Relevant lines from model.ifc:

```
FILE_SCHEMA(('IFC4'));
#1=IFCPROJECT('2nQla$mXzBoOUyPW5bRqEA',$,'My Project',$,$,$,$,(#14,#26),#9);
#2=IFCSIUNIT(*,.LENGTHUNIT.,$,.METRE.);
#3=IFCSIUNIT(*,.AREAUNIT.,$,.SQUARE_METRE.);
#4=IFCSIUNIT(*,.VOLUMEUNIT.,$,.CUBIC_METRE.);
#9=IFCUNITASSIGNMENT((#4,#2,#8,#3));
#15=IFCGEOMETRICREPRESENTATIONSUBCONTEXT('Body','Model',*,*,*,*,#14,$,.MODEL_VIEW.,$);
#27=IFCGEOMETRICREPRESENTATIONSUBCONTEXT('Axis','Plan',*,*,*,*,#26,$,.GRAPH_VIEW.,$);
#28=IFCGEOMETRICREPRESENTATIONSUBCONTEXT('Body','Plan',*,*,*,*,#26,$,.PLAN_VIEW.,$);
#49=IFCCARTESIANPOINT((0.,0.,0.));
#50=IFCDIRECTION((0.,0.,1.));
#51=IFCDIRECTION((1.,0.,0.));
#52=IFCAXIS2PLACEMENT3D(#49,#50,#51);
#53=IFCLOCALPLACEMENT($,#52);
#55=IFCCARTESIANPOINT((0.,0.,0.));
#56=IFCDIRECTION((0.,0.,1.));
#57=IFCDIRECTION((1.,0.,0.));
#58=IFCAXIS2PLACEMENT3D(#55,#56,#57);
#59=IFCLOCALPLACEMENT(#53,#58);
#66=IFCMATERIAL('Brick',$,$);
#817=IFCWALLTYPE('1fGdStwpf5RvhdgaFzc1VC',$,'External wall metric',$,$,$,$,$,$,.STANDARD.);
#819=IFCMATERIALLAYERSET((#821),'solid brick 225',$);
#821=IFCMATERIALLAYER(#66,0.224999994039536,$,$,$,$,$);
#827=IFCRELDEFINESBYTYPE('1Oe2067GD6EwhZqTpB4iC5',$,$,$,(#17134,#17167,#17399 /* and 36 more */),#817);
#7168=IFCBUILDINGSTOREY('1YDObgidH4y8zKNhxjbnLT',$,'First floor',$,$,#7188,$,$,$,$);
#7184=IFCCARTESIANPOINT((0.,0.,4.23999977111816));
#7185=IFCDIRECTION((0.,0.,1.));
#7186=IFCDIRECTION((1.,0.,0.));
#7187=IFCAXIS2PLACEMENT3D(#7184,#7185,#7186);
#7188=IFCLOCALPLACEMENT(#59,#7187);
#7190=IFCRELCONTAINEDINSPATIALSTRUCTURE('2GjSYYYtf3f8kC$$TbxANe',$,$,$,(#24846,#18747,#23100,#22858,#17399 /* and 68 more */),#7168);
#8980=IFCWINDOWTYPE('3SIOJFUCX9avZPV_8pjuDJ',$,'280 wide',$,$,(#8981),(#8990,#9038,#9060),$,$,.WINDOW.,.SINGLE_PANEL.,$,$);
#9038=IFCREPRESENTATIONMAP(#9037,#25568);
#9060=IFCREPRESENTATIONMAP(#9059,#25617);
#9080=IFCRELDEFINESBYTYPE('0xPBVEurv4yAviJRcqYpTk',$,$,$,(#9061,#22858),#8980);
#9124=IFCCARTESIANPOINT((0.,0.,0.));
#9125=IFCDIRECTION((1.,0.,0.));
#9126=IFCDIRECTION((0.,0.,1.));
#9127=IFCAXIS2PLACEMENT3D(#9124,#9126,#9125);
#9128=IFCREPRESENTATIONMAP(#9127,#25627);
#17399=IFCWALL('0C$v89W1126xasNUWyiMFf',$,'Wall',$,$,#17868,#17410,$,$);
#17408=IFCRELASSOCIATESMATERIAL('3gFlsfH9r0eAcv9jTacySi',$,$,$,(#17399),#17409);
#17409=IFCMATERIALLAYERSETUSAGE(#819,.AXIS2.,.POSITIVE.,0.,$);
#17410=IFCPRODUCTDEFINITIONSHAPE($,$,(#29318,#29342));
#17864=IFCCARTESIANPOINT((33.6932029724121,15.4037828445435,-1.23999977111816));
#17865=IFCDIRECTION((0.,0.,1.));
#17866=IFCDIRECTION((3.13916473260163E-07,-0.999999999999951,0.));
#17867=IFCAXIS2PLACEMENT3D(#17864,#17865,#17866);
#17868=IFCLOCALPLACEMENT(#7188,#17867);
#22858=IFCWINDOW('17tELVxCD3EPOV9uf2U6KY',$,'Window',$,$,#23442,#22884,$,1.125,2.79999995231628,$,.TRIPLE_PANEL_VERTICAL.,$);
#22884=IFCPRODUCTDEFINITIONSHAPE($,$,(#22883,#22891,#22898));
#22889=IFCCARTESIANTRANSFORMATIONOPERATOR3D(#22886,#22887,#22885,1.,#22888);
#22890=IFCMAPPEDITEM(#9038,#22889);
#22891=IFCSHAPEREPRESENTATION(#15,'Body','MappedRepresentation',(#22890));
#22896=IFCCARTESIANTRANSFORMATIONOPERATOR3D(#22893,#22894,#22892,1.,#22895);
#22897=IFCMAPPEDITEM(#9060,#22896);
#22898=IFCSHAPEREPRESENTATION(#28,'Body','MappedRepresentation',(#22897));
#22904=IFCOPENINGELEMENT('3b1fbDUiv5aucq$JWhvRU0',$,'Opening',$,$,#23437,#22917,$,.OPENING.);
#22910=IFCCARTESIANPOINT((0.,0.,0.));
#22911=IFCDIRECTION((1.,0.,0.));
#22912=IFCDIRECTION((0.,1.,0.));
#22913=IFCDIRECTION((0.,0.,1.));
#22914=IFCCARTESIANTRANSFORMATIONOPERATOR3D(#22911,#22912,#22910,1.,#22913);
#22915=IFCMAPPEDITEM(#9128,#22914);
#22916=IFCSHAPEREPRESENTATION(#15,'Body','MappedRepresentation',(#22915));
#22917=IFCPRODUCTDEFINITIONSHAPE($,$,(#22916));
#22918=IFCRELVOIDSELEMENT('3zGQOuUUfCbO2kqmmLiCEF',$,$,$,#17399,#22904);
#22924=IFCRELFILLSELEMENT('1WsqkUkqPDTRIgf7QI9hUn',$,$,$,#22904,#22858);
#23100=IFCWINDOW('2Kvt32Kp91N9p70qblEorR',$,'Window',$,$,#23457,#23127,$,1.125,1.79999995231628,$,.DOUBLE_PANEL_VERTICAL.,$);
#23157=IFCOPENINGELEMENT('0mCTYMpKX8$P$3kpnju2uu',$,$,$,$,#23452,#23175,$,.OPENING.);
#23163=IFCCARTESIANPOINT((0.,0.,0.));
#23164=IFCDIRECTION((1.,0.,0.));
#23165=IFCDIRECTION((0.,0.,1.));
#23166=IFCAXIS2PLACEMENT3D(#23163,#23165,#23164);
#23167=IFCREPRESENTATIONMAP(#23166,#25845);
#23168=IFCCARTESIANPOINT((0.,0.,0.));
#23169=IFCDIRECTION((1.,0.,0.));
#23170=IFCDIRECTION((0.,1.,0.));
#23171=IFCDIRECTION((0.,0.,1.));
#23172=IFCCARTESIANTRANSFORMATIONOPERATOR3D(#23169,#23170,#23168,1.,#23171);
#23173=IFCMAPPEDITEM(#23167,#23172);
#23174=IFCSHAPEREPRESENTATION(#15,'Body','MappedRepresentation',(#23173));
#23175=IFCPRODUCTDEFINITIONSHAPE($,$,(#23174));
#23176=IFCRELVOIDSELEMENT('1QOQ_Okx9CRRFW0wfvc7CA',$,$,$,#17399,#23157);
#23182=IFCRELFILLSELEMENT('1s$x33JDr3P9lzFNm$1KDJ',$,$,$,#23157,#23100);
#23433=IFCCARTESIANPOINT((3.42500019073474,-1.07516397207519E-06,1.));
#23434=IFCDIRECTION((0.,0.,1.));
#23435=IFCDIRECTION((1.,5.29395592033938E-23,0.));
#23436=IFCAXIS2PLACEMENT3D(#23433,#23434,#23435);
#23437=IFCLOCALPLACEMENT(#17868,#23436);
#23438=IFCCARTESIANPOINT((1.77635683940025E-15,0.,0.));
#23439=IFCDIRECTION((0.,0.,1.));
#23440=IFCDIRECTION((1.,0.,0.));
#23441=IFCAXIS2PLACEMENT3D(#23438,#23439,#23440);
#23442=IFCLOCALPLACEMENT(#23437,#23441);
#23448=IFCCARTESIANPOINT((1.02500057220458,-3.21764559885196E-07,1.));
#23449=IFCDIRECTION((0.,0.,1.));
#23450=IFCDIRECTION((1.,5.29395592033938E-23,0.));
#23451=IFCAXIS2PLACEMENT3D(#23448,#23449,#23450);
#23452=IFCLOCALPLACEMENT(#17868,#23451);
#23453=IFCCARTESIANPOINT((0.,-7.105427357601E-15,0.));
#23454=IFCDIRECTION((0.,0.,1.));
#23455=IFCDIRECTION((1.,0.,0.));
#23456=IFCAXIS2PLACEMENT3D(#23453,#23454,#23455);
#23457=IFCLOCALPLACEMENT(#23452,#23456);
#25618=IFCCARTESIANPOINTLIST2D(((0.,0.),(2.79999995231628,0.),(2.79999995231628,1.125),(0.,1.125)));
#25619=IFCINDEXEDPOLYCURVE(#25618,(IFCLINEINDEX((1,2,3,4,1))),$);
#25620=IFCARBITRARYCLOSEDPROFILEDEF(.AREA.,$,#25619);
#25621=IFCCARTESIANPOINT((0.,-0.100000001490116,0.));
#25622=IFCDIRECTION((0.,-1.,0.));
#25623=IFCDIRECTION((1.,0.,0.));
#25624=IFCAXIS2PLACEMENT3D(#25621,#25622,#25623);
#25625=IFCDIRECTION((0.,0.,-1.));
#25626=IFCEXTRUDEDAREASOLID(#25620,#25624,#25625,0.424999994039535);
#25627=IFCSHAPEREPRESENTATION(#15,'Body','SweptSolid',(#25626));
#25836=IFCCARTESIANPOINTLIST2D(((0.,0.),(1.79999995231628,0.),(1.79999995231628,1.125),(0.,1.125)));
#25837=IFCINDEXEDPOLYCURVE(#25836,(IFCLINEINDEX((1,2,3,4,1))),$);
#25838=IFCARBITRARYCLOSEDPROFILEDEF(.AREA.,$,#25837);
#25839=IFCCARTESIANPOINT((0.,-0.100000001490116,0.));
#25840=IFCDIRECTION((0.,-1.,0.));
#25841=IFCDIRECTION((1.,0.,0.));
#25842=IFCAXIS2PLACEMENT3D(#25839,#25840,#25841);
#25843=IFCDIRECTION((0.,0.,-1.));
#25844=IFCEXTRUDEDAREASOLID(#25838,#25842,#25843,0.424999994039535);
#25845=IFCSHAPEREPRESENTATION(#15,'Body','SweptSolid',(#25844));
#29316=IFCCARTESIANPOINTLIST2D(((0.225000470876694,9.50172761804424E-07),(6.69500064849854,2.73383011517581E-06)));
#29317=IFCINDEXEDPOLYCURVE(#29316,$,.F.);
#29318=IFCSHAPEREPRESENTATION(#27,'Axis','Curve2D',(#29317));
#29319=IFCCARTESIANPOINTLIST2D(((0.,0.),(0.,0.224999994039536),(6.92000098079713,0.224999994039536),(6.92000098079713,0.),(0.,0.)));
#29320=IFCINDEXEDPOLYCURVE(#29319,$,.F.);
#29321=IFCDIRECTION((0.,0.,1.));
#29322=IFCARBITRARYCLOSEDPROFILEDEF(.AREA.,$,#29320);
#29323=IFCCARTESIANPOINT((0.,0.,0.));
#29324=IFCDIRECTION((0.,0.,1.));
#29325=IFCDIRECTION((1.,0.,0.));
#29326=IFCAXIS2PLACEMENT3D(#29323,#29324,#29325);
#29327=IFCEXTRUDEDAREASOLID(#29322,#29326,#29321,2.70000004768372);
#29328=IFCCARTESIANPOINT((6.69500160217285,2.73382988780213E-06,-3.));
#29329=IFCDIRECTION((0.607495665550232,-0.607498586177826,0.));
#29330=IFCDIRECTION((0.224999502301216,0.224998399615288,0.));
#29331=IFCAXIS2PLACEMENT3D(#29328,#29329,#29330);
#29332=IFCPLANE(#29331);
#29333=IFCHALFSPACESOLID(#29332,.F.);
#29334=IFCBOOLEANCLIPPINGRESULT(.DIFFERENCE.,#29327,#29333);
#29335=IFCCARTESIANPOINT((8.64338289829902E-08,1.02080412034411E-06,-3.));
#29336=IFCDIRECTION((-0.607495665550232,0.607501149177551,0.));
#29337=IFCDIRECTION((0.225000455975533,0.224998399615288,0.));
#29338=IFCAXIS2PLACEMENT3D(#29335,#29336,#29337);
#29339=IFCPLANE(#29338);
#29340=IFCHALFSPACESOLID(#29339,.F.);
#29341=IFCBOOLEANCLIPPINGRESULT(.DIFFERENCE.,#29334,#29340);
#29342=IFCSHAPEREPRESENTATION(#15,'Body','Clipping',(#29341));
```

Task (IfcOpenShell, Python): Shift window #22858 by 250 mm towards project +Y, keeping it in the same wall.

```python
import ifcopenshell
import ifcopenshell.api.geometry
import ifcopenshell.util.placement
import ifcopenshell.util.unit

model = ifcopenshell.open("model.ifc")
unit_scale = ifcopenshell.util.unit.calculate_unit_scale(model)

window = model.by_guid("17tELVxCD3EPOV9uf2U6KY")
opening = window.FillsVoids[0].RelatingOpeningElement
wall = opening.VoidsElements[0].RelatingBuildingElement

wall_matrix = ifcopenshell.util.placement.get_local_placement(wall.ObjectPlacement)
shift = wall_matrix[:3, 0] * -0.25 / unit_scale
before = ifcopenshell.util.placement.get_local_placement(window.ObjectPlacement)[:3, 3].copy()

# The window is placed relative to its opening, so it follows when the opening moves.
matrix = ifcopenshell.util.placement.get_local_placement(opening.ObjectPlacement)
matrix[:3, 3] += shift
ifcopenshell.api.geometry.edit_object_placement(
    model, product=opening, matrix=matrix, is_si=False, should_transform_children=True
)

after = ifcopenshell.util.placement.get_local_placement(window.ObjectPlacement)[:3, 3]
print("window moved by", (after - before).round(3) + 0.0)

model.write("model-out.ifc")
```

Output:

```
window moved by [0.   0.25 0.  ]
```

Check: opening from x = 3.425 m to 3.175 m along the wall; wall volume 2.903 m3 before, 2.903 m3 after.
